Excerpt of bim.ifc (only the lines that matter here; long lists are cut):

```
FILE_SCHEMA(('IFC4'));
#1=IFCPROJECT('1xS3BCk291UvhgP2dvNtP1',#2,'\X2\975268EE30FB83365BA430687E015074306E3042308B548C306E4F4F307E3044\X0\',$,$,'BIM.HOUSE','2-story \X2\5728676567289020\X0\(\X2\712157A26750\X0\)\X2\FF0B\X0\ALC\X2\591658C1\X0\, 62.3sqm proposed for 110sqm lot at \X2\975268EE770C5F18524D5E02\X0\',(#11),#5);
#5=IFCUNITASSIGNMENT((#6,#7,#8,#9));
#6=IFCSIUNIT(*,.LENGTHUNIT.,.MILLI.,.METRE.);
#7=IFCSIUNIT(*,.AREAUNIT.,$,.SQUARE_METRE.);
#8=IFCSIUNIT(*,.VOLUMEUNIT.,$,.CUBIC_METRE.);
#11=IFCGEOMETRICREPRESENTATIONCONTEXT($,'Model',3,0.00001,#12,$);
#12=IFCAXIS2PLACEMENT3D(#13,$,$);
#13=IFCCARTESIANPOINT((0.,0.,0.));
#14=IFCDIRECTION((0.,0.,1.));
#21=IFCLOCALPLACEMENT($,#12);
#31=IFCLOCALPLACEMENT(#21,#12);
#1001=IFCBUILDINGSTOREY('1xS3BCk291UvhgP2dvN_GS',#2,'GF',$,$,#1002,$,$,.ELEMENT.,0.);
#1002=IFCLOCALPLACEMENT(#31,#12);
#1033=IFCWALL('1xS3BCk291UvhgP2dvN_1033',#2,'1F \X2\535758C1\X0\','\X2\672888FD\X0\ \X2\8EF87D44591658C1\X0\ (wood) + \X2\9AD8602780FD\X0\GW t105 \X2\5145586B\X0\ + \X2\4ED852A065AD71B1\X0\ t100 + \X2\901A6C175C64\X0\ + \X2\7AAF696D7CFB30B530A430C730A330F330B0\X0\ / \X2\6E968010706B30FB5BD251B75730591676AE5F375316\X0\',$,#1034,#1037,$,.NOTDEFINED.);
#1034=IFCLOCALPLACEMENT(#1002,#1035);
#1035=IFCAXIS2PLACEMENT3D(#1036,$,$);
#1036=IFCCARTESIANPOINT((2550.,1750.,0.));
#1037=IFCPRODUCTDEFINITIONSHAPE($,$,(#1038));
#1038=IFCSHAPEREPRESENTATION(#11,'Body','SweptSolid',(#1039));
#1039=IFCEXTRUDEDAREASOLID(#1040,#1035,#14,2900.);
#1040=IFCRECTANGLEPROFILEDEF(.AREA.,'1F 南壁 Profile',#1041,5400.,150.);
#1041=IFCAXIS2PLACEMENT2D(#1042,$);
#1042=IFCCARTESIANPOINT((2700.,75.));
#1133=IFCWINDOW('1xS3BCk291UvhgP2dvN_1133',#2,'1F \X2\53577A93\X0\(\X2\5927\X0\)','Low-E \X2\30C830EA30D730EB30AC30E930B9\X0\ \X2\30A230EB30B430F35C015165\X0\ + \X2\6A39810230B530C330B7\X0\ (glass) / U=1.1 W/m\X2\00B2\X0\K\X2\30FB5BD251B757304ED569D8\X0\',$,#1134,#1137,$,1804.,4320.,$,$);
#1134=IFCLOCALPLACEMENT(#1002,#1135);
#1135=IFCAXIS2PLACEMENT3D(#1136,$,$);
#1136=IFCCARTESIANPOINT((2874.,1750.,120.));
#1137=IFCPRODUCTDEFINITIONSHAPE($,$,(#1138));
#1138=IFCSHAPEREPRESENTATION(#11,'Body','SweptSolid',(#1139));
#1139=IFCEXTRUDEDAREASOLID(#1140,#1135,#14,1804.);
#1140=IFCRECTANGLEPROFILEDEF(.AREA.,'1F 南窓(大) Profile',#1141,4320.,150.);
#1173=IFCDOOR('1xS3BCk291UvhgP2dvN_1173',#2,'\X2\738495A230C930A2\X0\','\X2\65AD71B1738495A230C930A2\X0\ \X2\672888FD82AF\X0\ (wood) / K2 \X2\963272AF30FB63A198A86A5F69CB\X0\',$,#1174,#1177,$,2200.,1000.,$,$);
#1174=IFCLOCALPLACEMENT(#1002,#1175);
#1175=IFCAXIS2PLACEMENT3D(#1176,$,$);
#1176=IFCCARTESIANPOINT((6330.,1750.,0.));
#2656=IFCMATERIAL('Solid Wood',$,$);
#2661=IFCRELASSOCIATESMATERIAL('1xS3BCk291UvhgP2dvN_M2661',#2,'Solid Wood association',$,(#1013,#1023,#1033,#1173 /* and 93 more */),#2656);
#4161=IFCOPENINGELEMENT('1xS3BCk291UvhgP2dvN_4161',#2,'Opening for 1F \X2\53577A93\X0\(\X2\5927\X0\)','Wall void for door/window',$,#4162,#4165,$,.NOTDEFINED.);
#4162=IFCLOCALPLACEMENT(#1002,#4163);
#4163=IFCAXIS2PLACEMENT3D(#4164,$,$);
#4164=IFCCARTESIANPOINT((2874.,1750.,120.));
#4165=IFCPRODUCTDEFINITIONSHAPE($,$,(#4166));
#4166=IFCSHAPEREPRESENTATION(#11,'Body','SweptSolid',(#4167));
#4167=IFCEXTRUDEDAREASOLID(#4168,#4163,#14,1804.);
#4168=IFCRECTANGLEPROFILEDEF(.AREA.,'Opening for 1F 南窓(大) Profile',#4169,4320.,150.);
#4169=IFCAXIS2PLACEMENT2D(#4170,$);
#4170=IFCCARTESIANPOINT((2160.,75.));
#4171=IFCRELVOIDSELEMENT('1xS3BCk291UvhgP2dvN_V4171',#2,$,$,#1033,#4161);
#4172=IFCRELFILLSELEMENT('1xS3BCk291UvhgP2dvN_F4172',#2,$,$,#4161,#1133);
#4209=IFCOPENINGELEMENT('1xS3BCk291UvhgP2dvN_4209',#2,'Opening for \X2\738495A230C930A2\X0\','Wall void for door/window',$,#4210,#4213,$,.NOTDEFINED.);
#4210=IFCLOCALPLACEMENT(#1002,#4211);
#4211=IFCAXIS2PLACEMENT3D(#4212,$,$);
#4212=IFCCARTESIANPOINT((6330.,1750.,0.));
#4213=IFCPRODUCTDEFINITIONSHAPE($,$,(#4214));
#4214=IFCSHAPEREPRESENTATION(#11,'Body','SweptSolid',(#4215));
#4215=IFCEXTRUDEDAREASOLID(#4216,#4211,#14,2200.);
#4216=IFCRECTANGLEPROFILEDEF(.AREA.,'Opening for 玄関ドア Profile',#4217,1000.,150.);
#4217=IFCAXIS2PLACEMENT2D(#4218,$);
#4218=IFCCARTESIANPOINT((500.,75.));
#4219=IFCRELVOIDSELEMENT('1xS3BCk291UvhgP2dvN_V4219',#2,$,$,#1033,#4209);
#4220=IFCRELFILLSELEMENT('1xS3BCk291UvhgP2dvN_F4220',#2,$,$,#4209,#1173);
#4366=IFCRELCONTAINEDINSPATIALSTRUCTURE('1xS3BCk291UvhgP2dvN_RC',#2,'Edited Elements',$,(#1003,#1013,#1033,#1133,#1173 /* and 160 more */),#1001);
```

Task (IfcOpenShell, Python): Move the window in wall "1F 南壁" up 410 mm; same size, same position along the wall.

```python
import numpy as np
import ifcopenshell
import ifcopenshell.api.geometry
import ifcopenshell.util.placement
import ifcopenshell.util.unit

model = ifcopenshell.open("bim.ifc")
unit_scale = ifcopenshell.util.unit.calculate_unit_scale(model)

window = model.by_guid("1xS3BCk291UvhgP2dvN_1133")
opening = window.FillsVoids[0].RelatingOpeningElement
dz = 410.0

shift = np.array([0.0, 0.0, dz])
# The window is not placed relative to its opening, so move both.
for product in (opening, window):
    matrix = ifcopenshell.util.placement.get_local_placement(product.ObjectPlacement)
    matrix[:3, 3] += shift
    ifcopenshell.api.geometry.edit_object_placement(model, product=product, matrix=matrix, is_si=False)

print(f"moved by {dz * unit_scale:+.3f} m")

model.write("bim_updated.ifc")
```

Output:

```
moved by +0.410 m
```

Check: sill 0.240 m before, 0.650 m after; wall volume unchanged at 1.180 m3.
